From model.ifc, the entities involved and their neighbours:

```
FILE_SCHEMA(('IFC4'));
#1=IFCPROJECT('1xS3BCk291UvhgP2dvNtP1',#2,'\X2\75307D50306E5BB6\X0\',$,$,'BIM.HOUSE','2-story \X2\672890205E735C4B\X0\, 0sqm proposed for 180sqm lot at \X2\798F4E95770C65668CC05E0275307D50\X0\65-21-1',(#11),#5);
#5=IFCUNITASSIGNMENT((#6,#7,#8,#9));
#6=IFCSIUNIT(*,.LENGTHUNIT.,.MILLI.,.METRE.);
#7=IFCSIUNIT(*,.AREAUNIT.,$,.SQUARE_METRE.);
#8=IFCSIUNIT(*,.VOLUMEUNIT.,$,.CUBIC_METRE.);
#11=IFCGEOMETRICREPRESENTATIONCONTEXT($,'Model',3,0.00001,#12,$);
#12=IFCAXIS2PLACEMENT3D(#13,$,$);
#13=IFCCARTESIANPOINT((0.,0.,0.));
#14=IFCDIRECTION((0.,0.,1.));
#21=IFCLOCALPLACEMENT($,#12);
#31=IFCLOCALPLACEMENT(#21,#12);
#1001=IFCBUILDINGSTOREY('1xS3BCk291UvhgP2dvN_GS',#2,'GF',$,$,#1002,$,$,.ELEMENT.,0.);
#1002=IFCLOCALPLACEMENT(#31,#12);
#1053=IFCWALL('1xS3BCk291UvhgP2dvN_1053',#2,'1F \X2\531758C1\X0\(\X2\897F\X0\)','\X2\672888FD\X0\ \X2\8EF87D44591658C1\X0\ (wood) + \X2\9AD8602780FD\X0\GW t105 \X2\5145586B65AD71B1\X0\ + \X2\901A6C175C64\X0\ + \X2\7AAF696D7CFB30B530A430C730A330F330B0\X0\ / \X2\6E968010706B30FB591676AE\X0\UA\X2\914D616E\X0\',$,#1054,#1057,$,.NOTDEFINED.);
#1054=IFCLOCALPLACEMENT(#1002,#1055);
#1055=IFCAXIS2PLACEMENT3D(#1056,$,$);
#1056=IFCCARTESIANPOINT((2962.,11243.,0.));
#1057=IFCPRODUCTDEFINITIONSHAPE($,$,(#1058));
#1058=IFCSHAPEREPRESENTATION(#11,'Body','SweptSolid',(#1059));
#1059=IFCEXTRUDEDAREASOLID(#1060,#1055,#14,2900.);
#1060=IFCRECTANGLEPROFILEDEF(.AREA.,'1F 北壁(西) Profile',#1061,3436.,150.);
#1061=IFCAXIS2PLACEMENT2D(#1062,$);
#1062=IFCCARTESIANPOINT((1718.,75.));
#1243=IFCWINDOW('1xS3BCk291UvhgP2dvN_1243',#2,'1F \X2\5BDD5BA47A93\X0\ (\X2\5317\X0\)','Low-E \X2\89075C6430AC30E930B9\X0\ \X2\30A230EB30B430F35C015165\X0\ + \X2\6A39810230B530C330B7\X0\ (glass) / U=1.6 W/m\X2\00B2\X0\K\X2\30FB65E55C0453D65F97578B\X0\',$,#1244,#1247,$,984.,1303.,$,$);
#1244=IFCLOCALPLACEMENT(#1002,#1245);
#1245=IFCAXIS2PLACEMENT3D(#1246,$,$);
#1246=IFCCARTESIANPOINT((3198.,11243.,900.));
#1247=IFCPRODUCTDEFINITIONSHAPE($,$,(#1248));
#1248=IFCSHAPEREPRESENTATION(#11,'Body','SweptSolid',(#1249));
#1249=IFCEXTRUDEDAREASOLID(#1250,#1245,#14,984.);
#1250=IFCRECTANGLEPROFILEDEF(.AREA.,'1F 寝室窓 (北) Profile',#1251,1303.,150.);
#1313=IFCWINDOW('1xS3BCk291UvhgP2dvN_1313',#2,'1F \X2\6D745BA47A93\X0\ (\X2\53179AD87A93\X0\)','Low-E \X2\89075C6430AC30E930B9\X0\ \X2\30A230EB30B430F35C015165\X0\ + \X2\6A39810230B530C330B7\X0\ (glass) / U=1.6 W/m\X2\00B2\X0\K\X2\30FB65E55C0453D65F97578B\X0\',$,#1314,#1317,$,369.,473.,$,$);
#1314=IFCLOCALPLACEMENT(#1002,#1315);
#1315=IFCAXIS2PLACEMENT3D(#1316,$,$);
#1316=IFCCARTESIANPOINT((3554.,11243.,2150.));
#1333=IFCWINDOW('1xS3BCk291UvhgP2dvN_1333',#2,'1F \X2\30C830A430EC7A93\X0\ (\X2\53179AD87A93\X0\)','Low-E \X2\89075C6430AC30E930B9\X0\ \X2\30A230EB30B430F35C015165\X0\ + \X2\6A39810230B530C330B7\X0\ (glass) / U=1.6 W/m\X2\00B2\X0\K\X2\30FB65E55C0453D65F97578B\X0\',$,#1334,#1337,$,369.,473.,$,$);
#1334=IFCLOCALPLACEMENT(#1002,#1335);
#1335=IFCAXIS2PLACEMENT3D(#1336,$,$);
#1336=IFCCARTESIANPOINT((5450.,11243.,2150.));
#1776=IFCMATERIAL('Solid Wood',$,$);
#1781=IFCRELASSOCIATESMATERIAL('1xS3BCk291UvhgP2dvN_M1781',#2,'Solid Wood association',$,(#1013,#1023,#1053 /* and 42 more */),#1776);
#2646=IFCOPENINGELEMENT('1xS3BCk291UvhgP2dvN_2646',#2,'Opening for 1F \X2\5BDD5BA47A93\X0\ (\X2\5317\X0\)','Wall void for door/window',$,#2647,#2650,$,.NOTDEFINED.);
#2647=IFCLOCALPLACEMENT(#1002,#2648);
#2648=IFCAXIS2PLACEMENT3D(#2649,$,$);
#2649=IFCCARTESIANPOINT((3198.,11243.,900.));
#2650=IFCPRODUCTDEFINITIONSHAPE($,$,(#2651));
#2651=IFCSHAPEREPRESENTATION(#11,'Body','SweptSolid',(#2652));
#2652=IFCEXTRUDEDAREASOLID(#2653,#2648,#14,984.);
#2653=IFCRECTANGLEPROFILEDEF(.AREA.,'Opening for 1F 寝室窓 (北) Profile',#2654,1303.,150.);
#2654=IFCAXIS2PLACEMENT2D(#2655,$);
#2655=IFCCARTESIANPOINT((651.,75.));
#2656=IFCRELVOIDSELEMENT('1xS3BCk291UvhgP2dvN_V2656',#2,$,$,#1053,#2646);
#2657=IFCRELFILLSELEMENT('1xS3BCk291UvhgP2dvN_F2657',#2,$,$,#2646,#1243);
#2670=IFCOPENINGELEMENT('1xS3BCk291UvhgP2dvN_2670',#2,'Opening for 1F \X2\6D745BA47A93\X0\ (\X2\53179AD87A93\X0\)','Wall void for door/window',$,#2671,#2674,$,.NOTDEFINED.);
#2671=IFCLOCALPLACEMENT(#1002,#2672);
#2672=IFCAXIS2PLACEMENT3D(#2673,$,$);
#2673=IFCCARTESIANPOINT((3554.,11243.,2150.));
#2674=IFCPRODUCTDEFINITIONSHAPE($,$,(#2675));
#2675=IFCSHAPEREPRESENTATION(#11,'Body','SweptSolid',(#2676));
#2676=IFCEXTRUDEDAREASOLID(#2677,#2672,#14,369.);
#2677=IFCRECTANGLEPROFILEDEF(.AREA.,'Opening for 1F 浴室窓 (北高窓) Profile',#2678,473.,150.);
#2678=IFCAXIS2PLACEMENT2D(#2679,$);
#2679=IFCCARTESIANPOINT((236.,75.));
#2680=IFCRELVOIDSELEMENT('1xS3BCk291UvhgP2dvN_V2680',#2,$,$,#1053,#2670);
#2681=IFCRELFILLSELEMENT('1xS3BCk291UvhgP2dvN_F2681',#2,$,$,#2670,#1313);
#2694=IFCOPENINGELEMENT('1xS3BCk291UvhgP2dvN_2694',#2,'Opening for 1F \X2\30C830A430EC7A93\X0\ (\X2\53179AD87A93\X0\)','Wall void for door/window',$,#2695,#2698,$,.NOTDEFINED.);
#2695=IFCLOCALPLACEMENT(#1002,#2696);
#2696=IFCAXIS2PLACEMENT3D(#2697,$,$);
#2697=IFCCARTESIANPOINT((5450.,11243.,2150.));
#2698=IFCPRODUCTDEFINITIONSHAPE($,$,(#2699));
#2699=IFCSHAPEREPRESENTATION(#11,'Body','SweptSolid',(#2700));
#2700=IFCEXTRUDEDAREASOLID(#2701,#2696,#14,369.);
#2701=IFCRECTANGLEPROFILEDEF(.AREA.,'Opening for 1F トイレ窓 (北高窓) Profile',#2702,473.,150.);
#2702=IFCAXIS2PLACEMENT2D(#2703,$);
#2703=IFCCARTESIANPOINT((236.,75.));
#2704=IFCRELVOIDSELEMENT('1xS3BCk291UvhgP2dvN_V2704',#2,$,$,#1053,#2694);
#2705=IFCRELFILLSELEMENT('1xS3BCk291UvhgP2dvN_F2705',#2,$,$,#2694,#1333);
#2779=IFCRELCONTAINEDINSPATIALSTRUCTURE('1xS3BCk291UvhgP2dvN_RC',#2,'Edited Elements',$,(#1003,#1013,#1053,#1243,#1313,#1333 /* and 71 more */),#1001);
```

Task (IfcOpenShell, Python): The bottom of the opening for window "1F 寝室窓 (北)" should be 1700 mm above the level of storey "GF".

```python
import numpy as np
import ifcopenshell
import ifcopenshell.api.geometry
import ifcopenshell.geom
import ifcopenshell.util.element
import ifcopenshell.util.placement
import ifcopenshell.util.shape
import ifcopenshell.util.unit

model = ifcopenshell.open("model.ifc")
unit_scale = ifcopenshell.util.unit.calculate_unit_scale(model)

window = model.by_guid("1xS3BCk291UvhgP2dvN_1243")
opening = window.FillsVoids[0].RelatingOpeningElement
storey = ifcopenshell.util.element.get_container(window, ifc_class="IfcBuildingStorey")
level = ifcopenshell.util.placement.get_local_placement(storey.ObjectPlacement)[2, 3]

# The opening's origin need not be at the sill, so measure its lowest point.
shape = ifcopenshell.geom.create_shape(ifcopenshell.geom.settings(), opening)
bottom = ifcopenshell.util.shape.get_shape_bottom_elevation(shape, shape.geometry) / unit_scale
dz = level + 1.7 / unit_scale - bottom

shift = np.array([0.0, 0.0, dz])
# The window is not placed relative to its opening, so move both.
for product in (opening, window):
    matrix = ifcopenshell.util.placement.get_local_placement(product.ObjectPlacement)
    matrix[:3, 3] += shift
    ifcopenshell.api.geometry.edit_object_placement(model, product=product, matrix=matrix, is_si=False)

print(f"moved by {dz * unit_scale:+.3f} m")

model.write("model_edited.ifc")
```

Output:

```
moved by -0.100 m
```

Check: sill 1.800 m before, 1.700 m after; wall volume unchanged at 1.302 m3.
